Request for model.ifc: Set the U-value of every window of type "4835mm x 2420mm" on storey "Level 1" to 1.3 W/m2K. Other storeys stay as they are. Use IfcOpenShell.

First a look at what the model holds.

```python
import ifcopenshell
import ifcopenshell.util.element

model = ifcopenshell.open("model.ifc")
print(model.schema)
storey = next(s for s in model.by_type("IfcBuildingStorey") if s.Name == "Level 1")
windows = [e for e in ifcopenshell.util.element.get_decomposition(storey) if e.is_a("IfcWindow")]
seen = {}
for e in windows:
    element_type = ifcopenshell.util.element.get_type(e)
    key = (element_type.Name if element_type != e and element_type else None, ifcopenshell.util.element.get_pset(e, "Pset_WindowCommon", "ThermalTransmittance"))
    seen[key] = seen.get(key, 0) + 1
for (name, value), count in sorted(seen.items(), key=str):
    print(count, "x", name, "|", value)
```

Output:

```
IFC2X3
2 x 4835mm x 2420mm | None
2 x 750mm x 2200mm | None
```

```python
import ifcopenshell
import ifcopenshell.api.pset
import ifcopenshell.util.element

model = ifcopenshell.open("model.ifc")

storey = next(s for s in model.by_type("IfcBuildingStorey") if s.Name == "Level 1")
windows = [e for e in ifcopenshell.util.element.get_decomposition(storey) if e.is_a("IfcWindow")]

count = 0
for e in windows:
    element_type = ifcopenshell.util.element.get_type(e)
    if element_type in (None, e) or element_type.Name != "4835mm x 2420mm":
        continue
    # add_pset returns the element's existing set when there is one.
    pset = ifcopenshell.api.pset.add_pset(model, product=e, name="Pset_WindowCommon")
    ifcopenshell.api.pset.edit_pset(model, pset=pset, properties={"ThermalTransmittance": 1.3})
    count += 1

print(count, "windows updated")

model.write("model-out.ifc")
```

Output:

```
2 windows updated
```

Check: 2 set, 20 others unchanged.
